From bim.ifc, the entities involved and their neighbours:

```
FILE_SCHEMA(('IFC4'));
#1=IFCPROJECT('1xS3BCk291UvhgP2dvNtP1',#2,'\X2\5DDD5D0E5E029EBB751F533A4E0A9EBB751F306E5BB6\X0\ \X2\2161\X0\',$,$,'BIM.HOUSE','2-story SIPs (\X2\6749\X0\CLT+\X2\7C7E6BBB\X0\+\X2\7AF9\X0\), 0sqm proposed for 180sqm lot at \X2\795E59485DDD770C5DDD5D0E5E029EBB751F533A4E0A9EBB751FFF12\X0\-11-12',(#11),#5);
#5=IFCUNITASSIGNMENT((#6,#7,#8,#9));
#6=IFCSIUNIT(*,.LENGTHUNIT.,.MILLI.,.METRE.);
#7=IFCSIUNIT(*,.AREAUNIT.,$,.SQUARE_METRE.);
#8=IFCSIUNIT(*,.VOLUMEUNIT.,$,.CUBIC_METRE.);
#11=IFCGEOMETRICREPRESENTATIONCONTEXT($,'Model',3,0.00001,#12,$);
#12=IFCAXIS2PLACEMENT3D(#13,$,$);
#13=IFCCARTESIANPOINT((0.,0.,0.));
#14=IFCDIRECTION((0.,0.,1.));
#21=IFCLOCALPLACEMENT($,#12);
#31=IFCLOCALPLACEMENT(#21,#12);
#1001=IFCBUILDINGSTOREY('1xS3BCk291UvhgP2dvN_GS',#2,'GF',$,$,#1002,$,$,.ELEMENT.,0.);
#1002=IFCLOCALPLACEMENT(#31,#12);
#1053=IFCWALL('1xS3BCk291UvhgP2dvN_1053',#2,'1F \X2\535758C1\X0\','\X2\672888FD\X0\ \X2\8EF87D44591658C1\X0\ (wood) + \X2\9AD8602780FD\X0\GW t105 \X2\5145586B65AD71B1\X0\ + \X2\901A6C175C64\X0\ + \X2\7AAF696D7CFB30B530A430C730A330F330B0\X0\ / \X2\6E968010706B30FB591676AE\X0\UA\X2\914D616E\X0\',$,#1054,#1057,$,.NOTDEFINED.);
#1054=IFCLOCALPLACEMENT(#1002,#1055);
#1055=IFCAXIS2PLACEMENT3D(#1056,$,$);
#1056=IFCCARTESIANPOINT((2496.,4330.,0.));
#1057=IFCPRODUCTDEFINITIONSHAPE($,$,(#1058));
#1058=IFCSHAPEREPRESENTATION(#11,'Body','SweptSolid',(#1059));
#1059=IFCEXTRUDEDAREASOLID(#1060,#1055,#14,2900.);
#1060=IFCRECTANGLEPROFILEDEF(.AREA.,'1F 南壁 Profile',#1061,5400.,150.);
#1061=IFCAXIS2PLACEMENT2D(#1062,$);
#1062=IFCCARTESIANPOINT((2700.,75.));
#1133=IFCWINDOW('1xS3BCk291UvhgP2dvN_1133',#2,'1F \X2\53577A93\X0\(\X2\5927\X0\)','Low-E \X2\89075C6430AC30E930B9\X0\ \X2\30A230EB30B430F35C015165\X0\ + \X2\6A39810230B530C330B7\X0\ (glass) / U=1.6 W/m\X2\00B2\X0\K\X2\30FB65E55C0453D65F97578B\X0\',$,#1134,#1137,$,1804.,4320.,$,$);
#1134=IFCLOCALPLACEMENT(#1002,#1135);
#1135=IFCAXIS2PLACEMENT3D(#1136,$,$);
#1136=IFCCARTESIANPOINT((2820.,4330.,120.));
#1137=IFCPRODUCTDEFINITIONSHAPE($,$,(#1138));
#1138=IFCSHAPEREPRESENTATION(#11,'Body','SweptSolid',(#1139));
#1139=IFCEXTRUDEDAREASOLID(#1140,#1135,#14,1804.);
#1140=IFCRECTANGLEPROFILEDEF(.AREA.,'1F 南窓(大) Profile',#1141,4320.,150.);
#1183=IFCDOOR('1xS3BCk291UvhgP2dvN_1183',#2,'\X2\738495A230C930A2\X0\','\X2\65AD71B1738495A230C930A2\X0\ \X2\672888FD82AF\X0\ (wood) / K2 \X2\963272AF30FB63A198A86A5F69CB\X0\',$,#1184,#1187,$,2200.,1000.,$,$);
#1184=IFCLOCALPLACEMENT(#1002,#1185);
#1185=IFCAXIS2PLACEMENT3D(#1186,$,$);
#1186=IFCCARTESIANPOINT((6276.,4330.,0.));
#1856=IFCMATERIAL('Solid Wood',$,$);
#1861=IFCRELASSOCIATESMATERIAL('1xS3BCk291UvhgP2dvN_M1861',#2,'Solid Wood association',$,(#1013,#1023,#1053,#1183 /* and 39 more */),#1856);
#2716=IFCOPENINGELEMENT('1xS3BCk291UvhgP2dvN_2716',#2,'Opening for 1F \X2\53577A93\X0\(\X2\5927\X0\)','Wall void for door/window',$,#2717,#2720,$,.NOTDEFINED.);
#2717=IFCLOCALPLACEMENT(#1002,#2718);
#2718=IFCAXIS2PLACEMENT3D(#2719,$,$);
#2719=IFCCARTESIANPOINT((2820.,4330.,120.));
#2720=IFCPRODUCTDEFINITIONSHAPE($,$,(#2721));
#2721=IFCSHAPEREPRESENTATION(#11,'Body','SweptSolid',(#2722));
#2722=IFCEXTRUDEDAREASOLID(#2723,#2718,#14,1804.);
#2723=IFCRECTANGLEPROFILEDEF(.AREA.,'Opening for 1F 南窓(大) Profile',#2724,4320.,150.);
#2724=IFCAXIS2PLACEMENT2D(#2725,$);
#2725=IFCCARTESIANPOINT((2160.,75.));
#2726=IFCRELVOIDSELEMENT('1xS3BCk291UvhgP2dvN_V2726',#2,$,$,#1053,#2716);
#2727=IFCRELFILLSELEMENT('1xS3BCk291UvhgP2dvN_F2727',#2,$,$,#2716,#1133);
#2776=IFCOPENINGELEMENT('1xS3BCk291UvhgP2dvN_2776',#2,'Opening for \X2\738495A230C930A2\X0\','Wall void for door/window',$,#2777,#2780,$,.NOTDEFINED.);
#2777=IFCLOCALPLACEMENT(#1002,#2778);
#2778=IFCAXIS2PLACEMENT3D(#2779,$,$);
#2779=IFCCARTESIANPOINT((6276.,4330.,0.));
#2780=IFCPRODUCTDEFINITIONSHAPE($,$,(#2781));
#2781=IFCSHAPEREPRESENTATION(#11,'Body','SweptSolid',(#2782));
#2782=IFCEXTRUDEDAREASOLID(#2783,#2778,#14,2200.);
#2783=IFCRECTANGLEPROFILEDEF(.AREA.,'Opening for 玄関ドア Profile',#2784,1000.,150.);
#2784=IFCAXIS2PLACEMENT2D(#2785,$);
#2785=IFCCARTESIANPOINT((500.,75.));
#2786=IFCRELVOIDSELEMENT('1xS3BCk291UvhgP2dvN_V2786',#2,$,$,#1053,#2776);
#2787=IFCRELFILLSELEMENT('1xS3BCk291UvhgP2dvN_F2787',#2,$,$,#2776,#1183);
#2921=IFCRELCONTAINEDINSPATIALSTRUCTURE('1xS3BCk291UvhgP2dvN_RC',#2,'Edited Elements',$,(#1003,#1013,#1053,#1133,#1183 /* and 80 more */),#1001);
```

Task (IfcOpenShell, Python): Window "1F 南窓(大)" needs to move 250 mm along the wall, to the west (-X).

```python
import ifcopenshell
import ifcopenshell.api.geometry
import ifcopenshell.util.placement
import ifcopenshell.util.unit

model = ifcopenshell.open("bim.ifc")
unit_scale = ifcopenshell.util.unit.calculate_unit_scale(model)

window = model.by_id(1133)
opening = window.FillsVoids[0].RelatingOpeningElement
wall = opening.VoidsElements[0].RelatingBuildingElement

wall_matrix = ifcopenshell.util.placement.get_local_placement(wall.ObjectPlacement)
shift = wall_matrix[:3, 0] * -0.25 / unit_scale
before = ifcopenshell.util.placement.get_local_placement(window.ObjectPlacement)[:3, 3].copy()

# The window is not placed relative to its opening, so move both.
for product in (opening, window):
    matrix = ifcopenshell.util.placement.get_local_placement(product.ObjectPlacement)
    matrix[:3, 3] += shift
    ifcopenshell.api.geometry.edit_object_placement(model, product=product, matrix=matrix, is_si=False)

after = ifcopenshell.util.placement.get_local_placement(window.ObjectPlacement)[:3, 3]
print("window moved by", (after - before).round(3) + 0.0)

model.write("bim-out.ifc")
```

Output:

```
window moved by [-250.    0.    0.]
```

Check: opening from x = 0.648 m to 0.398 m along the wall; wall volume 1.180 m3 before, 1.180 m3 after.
